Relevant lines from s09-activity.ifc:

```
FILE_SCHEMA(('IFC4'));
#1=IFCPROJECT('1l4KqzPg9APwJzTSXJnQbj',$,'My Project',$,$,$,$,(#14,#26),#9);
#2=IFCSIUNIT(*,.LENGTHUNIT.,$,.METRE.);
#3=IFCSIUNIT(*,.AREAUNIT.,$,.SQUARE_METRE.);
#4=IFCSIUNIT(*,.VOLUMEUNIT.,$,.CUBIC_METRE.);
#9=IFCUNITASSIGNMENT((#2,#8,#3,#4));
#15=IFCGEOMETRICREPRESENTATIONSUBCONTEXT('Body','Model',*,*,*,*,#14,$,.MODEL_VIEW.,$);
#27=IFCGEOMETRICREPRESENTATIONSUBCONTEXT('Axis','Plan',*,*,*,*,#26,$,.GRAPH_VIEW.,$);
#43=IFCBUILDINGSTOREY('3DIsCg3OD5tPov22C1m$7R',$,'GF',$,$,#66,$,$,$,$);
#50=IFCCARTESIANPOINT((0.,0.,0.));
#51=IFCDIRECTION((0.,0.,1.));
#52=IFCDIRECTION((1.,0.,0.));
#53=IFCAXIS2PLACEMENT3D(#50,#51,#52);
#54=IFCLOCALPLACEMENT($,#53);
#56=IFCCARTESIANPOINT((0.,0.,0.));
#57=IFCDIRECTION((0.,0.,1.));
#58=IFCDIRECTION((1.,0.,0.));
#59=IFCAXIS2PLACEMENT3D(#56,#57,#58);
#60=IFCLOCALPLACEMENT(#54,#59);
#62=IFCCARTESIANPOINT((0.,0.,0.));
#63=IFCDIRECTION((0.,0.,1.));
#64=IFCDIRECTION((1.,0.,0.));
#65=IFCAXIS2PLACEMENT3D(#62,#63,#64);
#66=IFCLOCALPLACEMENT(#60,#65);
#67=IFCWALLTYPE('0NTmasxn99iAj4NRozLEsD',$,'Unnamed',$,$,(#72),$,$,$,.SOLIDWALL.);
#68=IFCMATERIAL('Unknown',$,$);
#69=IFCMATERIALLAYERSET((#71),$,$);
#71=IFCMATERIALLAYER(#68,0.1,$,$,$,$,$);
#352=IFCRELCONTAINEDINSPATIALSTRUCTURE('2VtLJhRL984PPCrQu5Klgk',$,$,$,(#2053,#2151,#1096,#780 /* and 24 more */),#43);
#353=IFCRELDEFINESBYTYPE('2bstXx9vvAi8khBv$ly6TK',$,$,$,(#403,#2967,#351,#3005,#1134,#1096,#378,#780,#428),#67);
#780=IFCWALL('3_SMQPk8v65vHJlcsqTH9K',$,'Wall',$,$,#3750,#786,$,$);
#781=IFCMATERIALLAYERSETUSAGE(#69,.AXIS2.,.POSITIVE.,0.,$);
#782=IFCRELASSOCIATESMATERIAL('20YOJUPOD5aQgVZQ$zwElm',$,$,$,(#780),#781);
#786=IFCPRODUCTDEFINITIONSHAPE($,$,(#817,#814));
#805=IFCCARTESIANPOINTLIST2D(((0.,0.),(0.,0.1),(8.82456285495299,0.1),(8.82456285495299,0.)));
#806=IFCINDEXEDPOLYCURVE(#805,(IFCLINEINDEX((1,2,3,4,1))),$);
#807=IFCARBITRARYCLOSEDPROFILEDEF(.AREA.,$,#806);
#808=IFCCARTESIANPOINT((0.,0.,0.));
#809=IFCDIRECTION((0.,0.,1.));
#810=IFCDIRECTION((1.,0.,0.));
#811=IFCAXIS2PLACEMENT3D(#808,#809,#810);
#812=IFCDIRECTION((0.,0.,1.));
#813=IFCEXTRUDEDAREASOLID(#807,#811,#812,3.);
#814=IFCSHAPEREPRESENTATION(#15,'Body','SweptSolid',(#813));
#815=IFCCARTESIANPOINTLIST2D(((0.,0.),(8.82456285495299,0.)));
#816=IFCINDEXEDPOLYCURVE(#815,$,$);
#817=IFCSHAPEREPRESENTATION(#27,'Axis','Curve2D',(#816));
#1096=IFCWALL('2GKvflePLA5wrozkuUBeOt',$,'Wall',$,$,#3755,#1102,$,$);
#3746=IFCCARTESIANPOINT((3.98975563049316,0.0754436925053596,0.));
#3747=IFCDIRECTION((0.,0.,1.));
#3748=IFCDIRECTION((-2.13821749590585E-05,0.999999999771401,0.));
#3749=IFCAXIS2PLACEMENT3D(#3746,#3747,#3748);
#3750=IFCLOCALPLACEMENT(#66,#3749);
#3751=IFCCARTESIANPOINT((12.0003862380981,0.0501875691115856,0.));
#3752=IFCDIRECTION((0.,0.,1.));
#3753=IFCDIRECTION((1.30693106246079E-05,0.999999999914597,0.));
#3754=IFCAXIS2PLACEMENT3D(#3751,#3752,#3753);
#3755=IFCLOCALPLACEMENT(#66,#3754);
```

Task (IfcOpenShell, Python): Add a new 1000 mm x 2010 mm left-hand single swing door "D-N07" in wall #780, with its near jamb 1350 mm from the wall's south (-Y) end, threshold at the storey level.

```python
import numpy as np
import ifcopenshell
import ifcopenshell.api.feature
import ifcopenshell.api.geometry
import ifcopenshell.api.root
import ifcopenshell.api.spatial
import ifcopenshell.geom
import ifcopenshell.util.element
import ifcopenshell.util.placement
import ifcopenshell.util.representation
import ifcopenshell.util.shape
import ifcopenshell.util.unit

model = ifcopenshell.open("s09-activity.ifc")
unit_scale = ifcopenshell.util.unit.calculate_unit_scale(model)
settings = ifcopenshell.geom.settings()


def volume(element):
    """Net volume in cubic metres, openings subtracted."""
    shape = ifcopenshell.geom.create_shape(settings, element)
    return ifcopenshell.util.shape.get_volume(shape.geometry)


wall = model.by_guid("3_SMQPk8v65vHJlcsqTH9K")
storey = ifcopenshell.util.element.get_container(wall, ifc_class="IfcBuildingStorey")
context = ifcopenshell.util.representation.get_context(model, "Model", "Body", "MODEL_VIEW")
before = volume(wall)

width, height, from_end, sill = 1, 2.01, 1.35, 0.0  # metres

# The wall runs along its own X axis, and the end named is its -X end.
wall_shape = ifcopenshell.geom.create_shape(settings, wall)
x, y, z = ifcopenshell.util.shape.get_vertices(wall_shape.geometry).T
start = x.min() + from_end
face, thickness = float(y.min()), float(y.max() - y.min())
wall_matrix = ifcopenshell.util.placement.get_local_placement(wall.ObjectPlacement)
level = ifcopenshell.util.placement.get_local_placement(storey.ObjectPlacement)[2, 3]


def in_wall(x, y):
    """Placement at x, y metres in the wall's axes, at sill height."""
    matrix = wall_matrix.copy()
    matrix[:, 3] = wall_matrix @ np.array([x / unit_scale, y / unit_scale, 0.0, 1.0])
    matrix[2, 3] = level + sill / unit_scale
    return matrix


# Opening: a box that overshoots both wall faces by 50 mm.
opening = ifcopenshell.api.root.create_entity(model, ifc_class="IfcOpeningElement", predefined_type="OPENING")
box = ifcopenshell.api.geometry.add_wall_representation(
    model, context=context, length=width, height=height, thickness=thickness + 0.1
)
ifcopenshell.api.geometry.assign_representation(model, product=opening, representation=box)
ifcopenshell.api.geometry.edit_object_placement(model, product=opening, matrix=in_wall(start, face - 0.05), is_si=False)
ifcopenshell.api.feature.add_feature(model, feature=opening, element=wall)

door = ifcopenshell.api.root.create_entity(model, ifc_class="IfcDoor", name="D-N07", predefined_type="DOOR")
door.OverallWidth, door.OverallHeight = width / unit_scale, height / unit_scale
door.OperationType = "SINGLE_SWING_LEFT"
body = ifcopenshell.api.geometry.add_door_representation(
    model,
    context=context,
    overall_width=door.OverallWidth,
    overall_height=door.OverallHeight,
    operation_type="SINGLE_SWING_LEFT",
    lining_properties={"LiningDepth": thickness / unit_scale, "ThresholdDepth": thickness / unit_scale},
)
ifcopenshell.api.geometry.assign_representation(model, product=door, representation=body)
ifcopenshell.api.spatial.assign_container(model, products=[door], relating_structure=storey)
ifcopenshell.api.feature.add_filling(model, opening=opening, element=door)

# The lining spans the wall, so the door starts at the wall face.
ifcopenshell.api.geometry.edit_object_placement(model, product=door, matrix=in_wall(start, face), is_si=False)

after = volume(wall)

print(f"wall volume {before:.3f} -> {after:.3f} m3")

model.write("s09-activity_v2.ifc")
```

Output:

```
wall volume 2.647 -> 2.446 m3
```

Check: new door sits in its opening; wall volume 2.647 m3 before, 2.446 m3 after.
